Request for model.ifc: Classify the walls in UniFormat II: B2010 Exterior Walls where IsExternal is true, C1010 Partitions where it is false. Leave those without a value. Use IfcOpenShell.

First a look at what the model holds.

```python
import ifcopenshell
import ifcopenshell.util.element

model = ifcopenshell.open("model.ifc")
print(model.schema)
print("classifications:", [c.Name for c in model.by_type("IfcClassification")])
values = [ifcopenshell.util.element.get_pset(e, "Pset_WallCommon", "IsExternal") for e in model.by_type("IfcWall")]
for value in (True, False, None):
    print("IsExternal", value, values.count(value))
```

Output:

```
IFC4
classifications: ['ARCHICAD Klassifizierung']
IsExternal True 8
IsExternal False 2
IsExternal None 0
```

```python
import ifcopenshell
import ifcopenshell.api.classification
import ifcopenshell.util.element

model = ifcopenshell.open("model.ifc")

system = ifcopenshell.api.classification.add_classification(model, classification="UniFormat II")

walls = model.by_type("IfcWall")
external = {e: ifcopenshell.util.element.get_pset(e, "Pset_WallCommon", "IsExternal") for e in walls}
for flag, code, name in ((True, "B2010", "Exterior Walls"), (False, "C1010", "Partitions")):
    products = [e for e in walls if external[e] is flag]
    ifcopenshell.api.classification.add_reference(
        model, products=products, classification=system, identification=code, name=name
    )
    print(code, len(products))

model.write("model_rev.ifc")
```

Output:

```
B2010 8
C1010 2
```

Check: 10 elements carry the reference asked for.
